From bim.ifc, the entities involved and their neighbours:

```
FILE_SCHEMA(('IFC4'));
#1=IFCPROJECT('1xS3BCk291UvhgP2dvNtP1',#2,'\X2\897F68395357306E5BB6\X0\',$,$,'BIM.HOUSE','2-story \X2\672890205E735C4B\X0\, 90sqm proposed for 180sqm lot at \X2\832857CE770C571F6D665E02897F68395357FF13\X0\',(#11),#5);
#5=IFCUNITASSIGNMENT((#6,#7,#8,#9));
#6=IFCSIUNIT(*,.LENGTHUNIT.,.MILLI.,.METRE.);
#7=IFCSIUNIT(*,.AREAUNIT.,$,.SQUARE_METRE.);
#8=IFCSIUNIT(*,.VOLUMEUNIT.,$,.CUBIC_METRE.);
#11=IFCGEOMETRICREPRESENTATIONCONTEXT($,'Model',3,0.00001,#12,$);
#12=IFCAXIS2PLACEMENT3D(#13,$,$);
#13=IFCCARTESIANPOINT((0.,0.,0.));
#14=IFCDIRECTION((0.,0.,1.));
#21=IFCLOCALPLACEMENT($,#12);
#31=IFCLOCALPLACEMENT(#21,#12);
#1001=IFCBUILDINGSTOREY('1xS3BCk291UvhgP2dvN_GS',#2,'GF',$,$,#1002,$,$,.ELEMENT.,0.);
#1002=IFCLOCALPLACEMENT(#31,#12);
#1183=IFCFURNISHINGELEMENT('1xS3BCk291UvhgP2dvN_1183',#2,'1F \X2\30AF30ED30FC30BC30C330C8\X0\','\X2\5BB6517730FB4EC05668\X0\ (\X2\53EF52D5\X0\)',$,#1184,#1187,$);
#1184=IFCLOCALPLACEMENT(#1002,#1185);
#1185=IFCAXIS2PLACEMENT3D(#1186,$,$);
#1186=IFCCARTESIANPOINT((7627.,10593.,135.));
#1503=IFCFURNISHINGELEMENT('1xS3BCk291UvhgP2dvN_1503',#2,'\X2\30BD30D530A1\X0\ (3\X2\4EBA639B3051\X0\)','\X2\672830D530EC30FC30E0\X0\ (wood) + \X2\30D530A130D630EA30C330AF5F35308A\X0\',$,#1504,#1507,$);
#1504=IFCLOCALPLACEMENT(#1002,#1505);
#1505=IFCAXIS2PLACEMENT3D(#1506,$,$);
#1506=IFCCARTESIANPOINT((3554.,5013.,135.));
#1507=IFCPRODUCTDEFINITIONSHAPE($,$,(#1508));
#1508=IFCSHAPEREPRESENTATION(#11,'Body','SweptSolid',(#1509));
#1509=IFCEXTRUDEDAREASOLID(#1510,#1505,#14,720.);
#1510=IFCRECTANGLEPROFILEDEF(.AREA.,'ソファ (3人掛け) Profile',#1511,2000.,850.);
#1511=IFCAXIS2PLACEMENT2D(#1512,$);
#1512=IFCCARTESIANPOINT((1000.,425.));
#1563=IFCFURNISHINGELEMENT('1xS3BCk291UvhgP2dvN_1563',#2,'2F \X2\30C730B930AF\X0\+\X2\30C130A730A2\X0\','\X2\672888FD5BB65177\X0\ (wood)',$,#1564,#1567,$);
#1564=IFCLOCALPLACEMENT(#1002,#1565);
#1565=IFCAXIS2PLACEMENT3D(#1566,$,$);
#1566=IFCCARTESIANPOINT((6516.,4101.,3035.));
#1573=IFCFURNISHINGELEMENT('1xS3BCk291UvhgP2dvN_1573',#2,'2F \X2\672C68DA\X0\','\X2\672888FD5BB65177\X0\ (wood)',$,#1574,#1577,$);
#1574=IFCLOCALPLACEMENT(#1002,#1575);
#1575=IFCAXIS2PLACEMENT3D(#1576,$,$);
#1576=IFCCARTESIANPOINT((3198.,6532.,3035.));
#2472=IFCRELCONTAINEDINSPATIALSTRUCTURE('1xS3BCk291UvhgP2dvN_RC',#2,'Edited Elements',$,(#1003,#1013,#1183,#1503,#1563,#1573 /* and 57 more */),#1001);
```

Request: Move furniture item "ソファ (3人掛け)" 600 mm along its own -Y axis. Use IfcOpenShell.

```python
import ifcopenshell
import ifcopenshell.api.geometry
import ifcopenshell.util.placement
import ifcopenshell.util.unit

model = ifcopenshell.open("bim.ifc")
unit_scale = ifcopenshell.util.unit.calculate_unit_scale(model)

item = model.by_id(1503)
matrix = ifcopenshell.util.placement.get_local_placement(item.ObjectPlacement)
matrix[:3, 3] -= matrix[:3, 1] * 0.6 / unit_scale
ifcopenshell.api.geometry.edit_object_placement(model, product=item, matrix=matrix, is_si=False)

print(ifcopenshell.util.placement.get_local_placement(item.ObjectPlacement).round(3) + 0.0)

model.write("bim_updated.ifc")
```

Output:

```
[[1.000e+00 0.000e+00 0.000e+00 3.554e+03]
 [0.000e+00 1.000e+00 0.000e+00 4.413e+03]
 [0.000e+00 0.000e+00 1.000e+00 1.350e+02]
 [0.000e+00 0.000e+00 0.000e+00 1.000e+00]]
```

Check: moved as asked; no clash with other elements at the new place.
